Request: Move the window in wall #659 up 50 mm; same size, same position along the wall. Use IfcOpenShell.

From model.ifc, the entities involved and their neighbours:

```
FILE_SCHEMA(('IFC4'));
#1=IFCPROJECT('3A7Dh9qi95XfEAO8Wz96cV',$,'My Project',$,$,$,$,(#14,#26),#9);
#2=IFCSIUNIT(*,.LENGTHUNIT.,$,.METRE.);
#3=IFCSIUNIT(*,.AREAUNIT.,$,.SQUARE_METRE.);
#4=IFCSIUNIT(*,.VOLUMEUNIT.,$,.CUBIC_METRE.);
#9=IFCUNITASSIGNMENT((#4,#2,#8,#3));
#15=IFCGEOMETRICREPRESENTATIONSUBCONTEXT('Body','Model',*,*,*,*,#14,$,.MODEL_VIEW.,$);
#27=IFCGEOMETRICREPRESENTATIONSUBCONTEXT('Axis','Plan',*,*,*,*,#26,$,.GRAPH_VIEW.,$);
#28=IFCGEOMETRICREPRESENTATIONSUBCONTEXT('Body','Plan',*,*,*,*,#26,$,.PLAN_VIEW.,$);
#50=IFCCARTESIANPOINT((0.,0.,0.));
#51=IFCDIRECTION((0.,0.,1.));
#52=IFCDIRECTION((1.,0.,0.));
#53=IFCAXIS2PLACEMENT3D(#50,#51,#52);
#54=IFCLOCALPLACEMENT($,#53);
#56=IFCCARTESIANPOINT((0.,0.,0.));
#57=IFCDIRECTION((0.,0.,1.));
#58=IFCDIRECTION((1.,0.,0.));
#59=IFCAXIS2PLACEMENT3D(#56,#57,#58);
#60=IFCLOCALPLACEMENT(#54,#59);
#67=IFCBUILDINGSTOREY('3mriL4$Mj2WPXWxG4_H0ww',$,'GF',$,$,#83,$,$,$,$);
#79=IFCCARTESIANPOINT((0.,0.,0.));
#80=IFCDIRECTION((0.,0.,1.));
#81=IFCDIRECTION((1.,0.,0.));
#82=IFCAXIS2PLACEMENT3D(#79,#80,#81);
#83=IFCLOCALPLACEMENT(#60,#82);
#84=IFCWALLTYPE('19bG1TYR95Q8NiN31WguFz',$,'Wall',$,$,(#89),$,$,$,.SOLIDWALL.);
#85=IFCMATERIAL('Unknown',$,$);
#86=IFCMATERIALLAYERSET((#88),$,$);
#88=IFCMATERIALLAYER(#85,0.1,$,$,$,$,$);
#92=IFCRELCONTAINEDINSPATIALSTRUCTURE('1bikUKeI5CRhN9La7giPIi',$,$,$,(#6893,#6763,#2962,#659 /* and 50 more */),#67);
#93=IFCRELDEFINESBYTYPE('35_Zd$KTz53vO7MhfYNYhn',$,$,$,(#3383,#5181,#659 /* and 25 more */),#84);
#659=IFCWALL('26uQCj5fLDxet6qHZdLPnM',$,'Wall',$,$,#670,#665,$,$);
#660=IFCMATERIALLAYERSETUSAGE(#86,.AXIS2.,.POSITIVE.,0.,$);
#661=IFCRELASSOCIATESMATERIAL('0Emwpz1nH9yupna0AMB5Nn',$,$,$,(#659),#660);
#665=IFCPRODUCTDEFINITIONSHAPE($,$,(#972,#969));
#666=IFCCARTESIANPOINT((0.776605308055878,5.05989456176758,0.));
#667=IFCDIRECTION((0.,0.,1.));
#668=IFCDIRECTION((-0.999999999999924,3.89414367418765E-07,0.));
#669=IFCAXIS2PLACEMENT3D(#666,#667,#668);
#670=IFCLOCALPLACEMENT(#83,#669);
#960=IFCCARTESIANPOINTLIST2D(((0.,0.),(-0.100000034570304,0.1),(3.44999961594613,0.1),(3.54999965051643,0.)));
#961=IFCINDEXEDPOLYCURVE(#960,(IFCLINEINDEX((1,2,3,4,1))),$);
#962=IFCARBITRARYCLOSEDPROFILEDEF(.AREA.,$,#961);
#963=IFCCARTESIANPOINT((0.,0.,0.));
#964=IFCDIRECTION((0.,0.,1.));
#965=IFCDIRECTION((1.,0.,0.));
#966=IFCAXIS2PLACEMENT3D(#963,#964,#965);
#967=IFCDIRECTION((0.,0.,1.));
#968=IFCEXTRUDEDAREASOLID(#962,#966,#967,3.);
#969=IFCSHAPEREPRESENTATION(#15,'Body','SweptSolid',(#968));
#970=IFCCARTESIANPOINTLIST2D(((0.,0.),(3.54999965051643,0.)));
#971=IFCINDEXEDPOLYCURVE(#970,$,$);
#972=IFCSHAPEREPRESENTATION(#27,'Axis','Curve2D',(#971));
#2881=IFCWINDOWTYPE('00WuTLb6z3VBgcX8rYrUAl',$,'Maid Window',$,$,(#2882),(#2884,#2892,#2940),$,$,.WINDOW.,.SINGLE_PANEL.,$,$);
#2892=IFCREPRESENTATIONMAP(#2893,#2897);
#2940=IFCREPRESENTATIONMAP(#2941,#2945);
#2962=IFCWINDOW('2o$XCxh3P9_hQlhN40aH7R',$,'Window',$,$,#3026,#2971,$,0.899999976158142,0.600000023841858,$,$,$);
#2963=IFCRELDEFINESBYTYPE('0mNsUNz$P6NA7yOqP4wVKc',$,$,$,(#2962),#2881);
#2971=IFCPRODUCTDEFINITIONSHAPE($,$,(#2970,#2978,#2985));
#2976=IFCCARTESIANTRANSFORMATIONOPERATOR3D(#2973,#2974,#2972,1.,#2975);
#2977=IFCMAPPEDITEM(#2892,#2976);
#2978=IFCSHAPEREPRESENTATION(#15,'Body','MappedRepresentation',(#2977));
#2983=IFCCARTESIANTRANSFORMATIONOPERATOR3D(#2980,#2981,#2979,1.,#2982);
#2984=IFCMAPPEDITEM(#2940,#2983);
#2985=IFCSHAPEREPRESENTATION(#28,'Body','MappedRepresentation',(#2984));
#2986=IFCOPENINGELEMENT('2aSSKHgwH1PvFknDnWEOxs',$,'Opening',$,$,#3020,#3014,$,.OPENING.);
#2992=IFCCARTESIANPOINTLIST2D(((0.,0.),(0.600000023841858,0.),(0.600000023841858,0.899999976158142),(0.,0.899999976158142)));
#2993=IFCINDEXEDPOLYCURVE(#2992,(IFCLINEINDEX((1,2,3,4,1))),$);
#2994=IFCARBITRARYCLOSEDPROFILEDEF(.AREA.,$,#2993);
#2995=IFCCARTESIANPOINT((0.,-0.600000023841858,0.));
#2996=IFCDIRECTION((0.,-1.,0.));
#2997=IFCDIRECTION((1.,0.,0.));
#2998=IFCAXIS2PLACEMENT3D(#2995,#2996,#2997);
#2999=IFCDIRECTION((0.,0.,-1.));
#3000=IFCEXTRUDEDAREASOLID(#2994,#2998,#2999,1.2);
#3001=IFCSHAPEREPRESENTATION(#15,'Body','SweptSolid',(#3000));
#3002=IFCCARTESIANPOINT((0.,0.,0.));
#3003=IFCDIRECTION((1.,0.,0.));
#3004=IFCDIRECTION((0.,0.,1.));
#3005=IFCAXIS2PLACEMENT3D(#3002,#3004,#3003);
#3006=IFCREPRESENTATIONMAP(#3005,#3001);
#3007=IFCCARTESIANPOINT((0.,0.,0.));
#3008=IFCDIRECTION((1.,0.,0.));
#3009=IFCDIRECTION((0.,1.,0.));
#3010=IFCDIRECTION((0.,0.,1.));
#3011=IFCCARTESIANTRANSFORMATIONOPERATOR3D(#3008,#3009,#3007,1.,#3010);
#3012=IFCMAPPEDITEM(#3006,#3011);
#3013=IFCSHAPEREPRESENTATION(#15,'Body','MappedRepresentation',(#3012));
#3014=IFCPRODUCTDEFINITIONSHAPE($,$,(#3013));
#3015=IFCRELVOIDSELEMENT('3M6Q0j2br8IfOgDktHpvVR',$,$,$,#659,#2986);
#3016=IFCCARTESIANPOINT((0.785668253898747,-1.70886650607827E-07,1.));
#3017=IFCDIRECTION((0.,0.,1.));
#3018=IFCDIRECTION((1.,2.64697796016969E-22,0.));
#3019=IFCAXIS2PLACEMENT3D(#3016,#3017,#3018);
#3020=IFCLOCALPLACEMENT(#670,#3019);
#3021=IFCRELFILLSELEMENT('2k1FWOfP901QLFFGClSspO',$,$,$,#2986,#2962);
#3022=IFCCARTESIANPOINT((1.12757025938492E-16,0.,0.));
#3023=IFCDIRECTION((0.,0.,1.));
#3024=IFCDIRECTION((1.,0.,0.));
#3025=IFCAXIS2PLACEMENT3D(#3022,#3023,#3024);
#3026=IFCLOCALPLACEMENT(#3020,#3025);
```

```python
import numpy as np
import ifcopenshell
import ifcopenshell.api.geometry
import ifcopenshell.util.placement
import ifcopenshell.util.unit

model = ifcopenshell.open("model.ifc")
unit_scale = ifcopenshell.util.unit.calculate_unit_scale(model)

window = model.by_guid("2o$XCxh3P9_hQlhN40aH7R")
opening = window.FillsVoids[0].RelatingOpeningElement
dz = 0.05

shift = np.array([0.0, 0.0, dz])
# The window is placed relative to its opening, so it follows when the opening moves.
matrix = ifcopenshell.util.placement.get_local_placement(opening.ObjectPlacement)
matrix[:3, 3] += shift
ifcopenshell.api.geometry.edit_object_placement(
    model, product=opening, matrix=matrix, is_si=False, should_transform_children=True
)

print(f"moved by {dz * unit_scale:+.3f} m")

model.write("model_rev.ifc")
```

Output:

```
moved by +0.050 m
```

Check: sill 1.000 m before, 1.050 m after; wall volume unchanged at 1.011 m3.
